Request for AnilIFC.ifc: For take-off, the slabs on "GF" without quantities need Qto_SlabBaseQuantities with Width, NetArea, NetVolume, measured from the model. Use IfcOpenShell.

First a look at what the model holds.

```python
import ifcopenshell
import ifcopenshell.util.element
import ifcopenshell.util.unit

model = ifcopenshell.open("AnilIFC.ifc")
print(model.schema)
for unit_type in ("LENGTHUNIT", "AREAUNIT", "VOLUMEUNIT"):
    print(unit_type, ifcopenshell.util.unit.calculate_unit_scale(model, unit_type))
storey = next(s for s in model.by_type("IfcBuildingStorey") if s.Name == "GF")
slabs = [e for e in ifcopenshell.util.element.get_decomposition(storey) if e.is_a("IfcSlab")]
for e in sorted(slabs, key=lambda e: e.id()):
    print(e.id(), e.is_a(), e.Name, list(ifcopenshell.util.element.get_psets(e, qtos_only=True)), sep=" | ")
```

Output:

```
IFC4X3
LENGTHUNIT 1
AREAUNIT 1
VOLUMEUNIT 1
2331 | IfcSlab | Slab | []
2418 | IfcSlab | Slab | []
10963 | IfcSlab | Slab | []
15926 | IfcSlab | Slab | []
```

```python
import ifcopenshell
import ifcopenshell.api.pset
import ifcopenshell.geom
import ifcopenshell.util.element
import ifcopenshell.util.shape
import ifcopenshell.util.unit

model = ifcopenshell.open("AnilIFC.ifc")
unit_scale = ifcopenshell.util.unit.calculate_unit_scale(model)
area_scale = ifcopenshell.util.unit.calculate_unit_scale(model, "AREAUNIT")
volume_scale = ifcopenshell.util.unit.calculate_unit_scale(model, "VOLUMEUNIT")
settings = ifcopenshell.geom.settings()

storey = next(s for s in model.by_type("IfcBuildingStorey") if s.Name == "GF")
slabs = [e for e in ifcopenshell.util.element.get_decomposition(storey) if e.is_a("IfcSlab")]

for e in sorted(slabs, key=lambda e: e.id()):
    if ifcopenshell.util.element.get_psets(e, qtos_only=True, should_inherit=False):
        continue
    # Geometry comes back in metres, in the element's own axes.
    shape = ifcopenshell.geom.create_shape(settings, e)
    values = {
        "Width": ifcopenshell.util.shape.get_z(shape.geometry) / unit_scale,
        "NetArea": ifcopenshell.util.shape.get_footprint_area(shape.geometry) / area_scale,
        "NetVolume": ifcopenshell.util.shape.get_volume(shape.geometry) / volume_scale,
    }
    qto = ifcopenshell.api.pset.add_qto(model, product=e, name="Qto_SlabBaseQuantities")
    ifcopenshell.api.pset.edit_qto(model, qto=qto, properties=values)
    print(e.id(), {k: round(v, 3) for k, v in values.items()})

model.write("AnilIFC_updated.ifc")
```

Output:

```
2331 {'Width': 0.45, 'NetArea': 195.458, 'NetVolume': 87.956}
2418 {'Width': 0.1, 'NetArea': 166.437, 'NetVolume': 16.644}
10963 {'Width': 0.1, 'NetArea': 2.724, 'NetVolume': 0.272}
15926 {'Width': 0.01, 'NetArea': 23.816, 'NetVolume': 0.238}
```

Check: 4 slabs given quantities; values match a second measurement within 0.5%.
